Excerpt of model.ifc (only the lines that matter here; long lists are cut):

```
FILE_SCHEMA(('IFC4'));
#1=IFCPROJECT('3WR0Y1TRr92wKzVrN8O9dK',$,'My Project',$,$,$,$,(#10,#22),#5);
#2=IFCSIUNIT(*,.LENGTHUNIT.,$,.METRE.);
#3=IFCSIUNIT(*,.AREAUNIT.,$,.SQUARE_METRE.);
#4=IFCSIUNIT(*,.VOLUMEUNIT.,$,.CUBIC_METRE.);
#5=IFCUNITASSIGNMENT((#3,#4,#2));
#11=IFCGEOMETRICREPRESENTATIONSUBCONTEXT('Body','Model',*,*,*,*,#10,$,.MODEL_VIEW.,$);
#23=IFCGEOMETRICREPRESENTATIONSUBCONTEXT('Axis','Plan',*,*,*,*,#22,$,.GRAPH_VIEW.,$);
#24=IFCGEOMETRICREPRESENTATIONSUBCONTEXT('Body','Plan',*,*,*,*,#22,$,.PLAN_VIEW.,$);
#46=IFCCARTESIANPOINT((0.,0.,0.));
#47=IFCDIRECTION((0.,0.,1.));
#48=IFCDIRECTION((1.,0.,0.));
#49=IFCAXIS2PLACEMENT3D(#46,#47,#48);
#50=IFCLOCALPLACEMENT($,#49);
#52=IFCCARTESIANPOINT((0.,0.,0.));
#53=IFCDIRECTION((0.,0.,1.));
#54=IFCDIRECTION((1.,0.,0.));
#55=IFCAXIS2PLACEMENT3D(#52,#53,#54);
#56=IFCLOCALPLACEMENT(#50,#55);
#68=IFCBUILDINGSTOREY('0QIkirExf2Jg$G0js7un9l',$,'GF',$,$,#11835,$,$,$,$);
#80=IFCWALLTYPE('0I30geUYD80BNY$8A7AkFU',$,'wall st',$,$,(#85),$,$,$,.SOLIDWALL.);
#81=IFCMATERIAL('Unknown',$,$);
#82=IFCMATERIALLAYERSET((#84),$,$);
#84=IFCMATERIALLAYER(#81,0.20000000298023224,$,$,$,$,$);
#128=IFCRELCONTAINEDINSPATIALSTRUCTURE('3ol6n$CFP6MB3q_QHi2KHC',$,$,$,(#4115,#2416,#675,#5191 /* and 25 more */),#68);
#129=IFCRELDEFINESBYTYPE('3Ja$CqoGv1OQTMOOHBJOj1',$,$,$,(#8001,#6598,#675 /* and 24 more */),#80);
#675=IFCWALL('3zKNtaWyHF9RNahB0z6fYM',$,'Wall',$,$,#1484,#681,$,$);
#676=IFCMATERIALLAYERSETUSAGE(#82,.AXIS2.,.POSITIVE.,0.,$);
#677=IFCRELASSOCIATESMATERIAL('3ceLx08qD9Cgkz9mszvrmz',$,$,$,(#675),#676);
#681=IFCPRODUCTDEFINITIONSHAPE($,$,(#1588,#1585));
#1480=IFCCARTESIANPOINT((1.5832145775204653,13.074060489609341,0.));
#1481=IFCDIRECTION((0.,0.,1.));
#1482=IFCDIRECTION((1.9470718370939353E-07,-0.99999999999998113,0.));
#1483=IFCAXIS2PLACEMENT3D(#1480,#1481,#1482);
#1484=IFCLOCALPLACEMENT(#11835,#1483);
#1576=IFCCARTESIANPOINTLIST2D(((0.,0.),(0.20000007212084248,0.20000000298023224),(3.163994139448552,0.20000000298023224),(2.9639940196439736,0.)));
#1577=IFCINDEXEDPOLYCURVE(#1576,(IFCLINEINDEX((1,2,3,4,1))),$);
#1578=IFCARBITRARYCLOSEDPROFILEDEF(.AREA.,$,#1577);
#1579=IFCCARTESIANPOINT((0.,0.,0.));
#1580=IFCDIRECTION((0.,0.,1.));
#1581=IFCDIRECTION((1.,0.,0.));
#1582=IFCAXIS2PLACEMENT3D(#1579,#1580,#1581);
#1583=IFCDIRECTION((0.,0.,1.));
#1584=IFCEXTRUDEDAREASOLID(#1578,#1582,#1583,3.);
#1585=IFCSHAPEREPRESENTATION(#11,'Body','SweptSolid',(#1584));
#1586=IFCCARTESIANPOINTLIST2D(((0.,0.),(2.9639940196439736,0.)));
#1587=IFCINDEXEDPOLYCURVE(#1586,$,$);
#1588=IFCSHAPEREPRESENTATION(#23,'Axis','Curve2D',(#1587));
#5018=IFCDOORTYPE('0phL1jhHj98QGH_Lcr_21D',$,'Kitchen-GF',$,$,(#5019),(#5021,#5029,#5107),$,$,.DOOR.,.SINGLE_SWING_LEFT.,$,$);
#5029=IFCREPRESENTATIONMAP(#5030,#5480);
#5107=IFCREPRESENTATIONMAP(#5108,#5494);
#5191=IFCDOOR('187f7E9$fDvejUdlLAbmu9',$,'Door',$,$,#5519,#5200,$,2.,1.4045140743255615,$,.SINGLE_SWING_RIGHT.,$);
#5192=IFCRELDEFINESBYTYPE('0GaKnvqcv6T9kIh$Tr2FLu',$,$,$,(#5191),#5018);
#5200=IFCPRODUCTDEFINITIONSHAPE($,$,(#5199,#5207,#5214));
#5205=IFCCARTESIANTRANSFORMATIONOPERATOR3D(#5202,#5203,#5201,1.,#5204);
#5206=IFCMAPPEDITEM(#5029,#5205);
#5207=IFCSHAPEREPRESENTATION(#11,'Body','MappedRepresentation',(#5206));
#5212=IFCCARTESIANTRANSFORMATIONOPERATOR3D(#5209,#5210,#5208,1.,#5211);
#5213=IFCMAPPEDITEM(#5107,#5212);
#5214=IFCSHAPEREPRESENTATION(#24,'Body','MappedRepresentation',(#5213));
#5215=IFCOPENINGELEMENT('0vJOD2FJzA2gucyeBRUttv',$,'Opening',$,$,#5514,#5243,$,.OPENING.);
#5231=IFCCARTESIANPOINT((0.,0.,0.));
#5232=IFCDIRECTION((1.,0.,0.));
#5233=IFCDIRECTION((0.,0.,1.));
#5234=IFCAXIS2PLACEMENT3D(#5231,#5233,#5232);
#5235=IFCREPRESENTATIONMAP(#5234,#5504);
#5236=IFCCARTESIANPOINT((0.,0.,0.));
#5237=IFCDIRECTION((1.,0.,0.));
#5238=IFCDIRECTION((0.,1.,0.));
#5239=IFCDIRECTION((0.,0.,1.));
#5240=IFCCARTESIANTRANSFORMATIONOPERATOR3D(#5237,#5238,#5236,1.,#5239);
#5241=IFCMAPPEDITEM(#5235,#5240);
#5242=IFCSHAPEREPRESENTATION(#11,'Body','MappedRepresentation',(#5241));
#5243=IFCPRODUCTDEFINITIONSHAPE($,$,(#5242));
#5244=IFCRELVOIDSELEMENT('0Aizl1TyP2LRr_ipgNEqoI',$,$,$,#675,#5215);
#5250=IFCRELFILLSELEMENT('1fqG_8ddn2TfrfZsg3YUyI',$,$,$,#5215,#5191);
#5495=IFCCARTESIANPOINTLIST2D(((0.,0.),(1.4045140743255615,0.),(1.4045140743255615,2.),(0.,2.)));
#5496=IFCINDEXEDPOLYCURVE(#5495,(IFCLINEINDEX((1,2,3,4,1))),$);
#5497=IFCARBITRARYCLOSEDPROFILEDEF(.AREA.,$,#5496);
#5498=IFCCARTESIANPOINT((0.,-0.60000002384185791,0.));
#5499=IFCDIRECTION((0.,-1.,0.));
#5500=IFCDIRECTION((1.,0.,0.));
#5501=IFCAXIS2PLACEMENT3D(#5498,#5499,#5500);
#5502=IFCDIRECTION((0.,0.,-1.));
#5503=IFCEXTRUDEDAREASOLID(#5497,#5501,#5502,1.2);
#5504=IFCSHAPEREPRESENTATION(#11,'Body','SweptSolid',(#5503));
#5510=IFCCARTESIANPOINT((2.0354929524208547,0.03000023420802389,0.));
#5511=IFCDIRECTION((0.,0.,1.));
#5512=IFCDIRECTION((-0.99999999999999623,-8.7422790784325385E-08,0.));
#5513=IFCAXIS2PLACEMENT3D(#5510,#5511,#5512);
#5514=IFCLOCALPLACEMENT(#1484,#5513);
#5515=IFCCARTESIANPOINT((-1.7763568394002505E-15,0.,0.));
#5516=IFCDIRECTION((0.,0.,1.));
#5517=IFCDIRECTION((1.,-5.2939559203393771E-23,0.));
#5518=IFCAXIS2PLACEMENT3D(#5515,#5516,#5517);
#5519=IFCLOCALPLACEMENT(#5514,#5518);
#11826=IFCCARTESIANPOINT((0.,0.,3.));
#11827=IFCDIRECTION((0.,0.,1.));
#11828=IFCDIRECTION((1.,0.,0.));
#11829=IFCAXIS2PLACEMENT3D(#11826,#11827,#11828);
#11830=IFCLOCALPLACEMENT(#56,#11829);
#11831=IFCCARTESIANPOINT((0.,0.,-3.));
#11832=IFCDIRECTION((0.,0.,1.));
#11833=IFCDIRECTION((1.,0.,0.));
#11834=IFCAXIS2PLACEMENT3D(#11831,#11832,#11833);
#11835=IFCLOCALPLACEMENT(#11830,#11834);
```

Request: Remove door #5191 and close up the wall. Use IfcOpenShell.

```python
import ifcopenshell
import ifcopenshell.api.feature
import ifcopenshell.api.root
import ifcopenshell.geom
import ifcopenshell.util.shape

model = ifcopenshell.open("model.ifc")
settings = ifcopenshell.geom.settings()


def volume(element):
    """Net volume in cubic metres, openings subtracted."""
    shape = ifcopenshell.geom.create_shape(settings, element)
    return ifcopenshell.util.shape.get_volume(shape.geometry)


door = model.by_guid("187f7E9$fDvejUdlLAbmu9")
opening = door.FillsVoids[0].RelatingOpeningElement
wall = opening.VoidsElements[0].RelatingBuildingElement
before = volume(wall)

ifcopenshell.api.root.remove_product(model, product=door)
ifcopenshell.api.feature.remove_feature(model, feature=opening)

after = volume(wall)

print(f"wall volume {before:.3f} -> {after:.3f} m3")

model.write("model_edited.ifc")
```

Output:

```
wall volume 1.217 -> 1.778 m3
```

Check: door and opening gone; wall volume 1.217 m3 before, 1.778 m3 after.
